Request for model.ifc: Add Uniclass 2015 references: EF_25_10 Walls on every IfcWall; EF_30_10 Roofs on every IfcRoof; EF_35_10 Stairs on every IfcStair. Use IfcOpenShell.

First a look at what the model holds.

```python
import ifcopenshell

model = ifcopenshell.open("model.ifc")
print(model.schema)
print("classifications:", [c.Name for c in model.by_type("IfcClassification")])
for ifc_class in ("IfcDoor", "IfcRoof", "IfcStair", "IfcWall", "IfcWindow"):
    print(ifc_class, len(model.by_type(ifc_class)))
```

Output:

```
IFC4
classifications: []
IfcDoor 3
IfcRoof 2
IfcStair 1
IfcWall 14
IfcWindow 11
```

```python
import ifcopenshell
import ifcopenshell.api.classification

model = ifcopenshell.open("model.ifc")

system = ifcopenshell.api.classification.add_classification(model, classification="Uniclass 2015")

codes = {
    "IfcWall": ("EF_25_10", "Walls"),
    "IfcRoof": ("EF_30_10", "Roofs"),
    "IfcStair": ("EF_35_10", "Stairs"),
}
for ifc_class, (code, name) in codes.items():
    products = model.by_type(ifc_class)
    ifcopenshell.api.classification.add_reference(
        model, products=products, classification=system, identification=code, name=name
    )
    print(code, len(products))

model.write("model_edited.ifc")
```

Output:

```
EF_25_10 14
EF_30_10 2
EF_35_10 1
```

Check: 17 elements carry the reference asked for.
